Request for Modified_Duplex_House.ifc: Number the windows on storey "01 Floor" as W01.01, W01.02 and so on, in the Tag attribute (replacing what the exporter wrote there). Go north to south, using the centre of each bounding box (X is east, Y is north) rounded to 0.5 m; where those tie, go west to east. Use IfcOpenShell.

First a look at what the model holds.

```python
import ifcopenshell
import ifcopenshell.util.element
import ifcopenshell.util.placement

model = ifcopenshell.open("Modified_Duplex_House.ifc")
print(model.schema)
storey = next(s for s in model.by_type("IfcBuildingStorey") if s.Name == "01 Floor")
windows = [e for e in ifcopenshell.util.element.get_decomposition(storey) if e.is_a("IfcWindow")]
for e in sorted(windows, key=lambda e: e.id()):
    origin = ifcopenshell.util.placement.get_local_placement(e.ObjectPlacement)[:3, 3]
    print(e.id(), e.Tag, e.Name, origin.round(2) + 0.0, sep=" | ")
```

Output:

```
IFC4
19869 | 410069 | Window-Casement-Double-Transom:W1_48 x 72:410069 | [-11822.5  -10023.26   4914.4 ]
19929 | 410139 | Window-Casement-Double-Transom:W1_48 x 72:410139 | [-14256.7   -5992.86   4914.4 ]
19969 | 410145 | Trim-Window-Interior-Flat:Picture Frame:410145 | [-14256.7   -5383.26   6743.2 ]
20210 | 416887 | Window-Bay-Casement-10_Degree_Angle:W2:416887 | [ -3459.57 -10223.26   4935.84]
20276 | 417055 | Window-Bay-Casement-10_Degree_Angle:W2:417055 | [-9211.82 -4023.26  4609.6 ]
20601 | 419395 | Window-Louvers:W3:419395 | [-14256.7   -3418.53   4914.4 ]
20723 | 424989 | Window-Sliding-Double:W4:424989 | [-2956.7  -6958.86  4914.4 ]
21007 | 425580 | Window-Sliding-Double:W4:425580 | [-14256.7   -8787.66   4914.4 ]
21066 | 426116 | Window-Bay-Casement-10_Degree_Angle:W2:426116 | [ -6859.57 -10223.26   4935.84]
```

```python
import ifcopenshell
import ifcopenshell.geom
import ifcopenshell.util.element
import ifcopenshell.util.shape

model = ifcopenshell.open("Modified_Duplex_House.ifc")
settings = ifcopenshell.geom.settings()
settings.set("use-world-coords", True)


def centre(element):
    shape = ifcopenshell.geom.create_shape(settings, element)
    return ifcopenshell.util.shape.get_bbox_centroid(shape.geometry)


storey = next(s for s in model.by_type("IfcBuildingStorey") if s.Name == "01 Floor")
windows = [e for e in ifcopenshell.util.element.get_decomposition(storey) if e.is_a("IfcWindow")]

# Insertion points can sit at a corner or the storey origin, so sort by the geometry (in metres).
centres = {e: centre(e) for e in windows}
windows.sort(key=lambda e: (-round(centres[e][1] / 0.5), centres[e][0]))

for i, e in enumerate(windows, start=1):
    number = f"W01.{i:02d}"
    e.Tag = number
    print(e.id(), number)

model.write("Modified_Duplex_House_edited.ifc")
```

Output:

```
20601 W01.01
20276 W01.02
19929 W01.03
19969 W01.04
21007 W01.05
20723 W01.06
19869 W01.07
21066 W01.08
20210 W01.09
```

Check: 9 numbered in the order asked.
